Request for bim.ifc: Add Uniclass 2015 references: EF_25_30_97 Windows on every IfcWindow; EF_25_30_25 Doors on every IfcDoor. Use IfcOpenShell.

First a look at what the model holds.

```python
import ifcopenshell

model = ifcopenshell.open("bim.ifc")
print(model.schema)
print("classifications:", [c.Name for c in model.by_type("IfcClassification")])
for ifc_class in ("IfcDoor", "IfcRoof", "IfcStair", "IfcWall", "IfcWindow"):
    print(ifc_class, len(model.by_type(ifc_class)))
```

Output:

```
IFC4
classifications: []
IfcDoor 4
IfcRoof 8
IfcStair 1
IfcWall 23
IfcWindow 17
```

```python
import ifcopenshell
import ifcopenshell.api.classification

model = ifcopenshell.open("bim.ifc")

system = ifcopenshell.api.classification.add_classification(model, classification="Uniclass 2015")

codes = {
    "IfcWindow": ("EF_25_30_97", "Windows"),
    "IfcDoor": ("EF_25_30_25", "Doors"),
}
for ifc_class, (code, name) in codes.items():
    products = model.by_type(ifc_class)
    ifcopenshell.api.classification.add_reference(
        model, products=products, classification=system, identification=code, name=name
    )
    print(code, len(products))

model.write("bim_updated.ifc")
```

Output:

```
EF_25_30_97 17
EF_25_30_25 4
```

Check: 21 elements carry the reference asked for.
